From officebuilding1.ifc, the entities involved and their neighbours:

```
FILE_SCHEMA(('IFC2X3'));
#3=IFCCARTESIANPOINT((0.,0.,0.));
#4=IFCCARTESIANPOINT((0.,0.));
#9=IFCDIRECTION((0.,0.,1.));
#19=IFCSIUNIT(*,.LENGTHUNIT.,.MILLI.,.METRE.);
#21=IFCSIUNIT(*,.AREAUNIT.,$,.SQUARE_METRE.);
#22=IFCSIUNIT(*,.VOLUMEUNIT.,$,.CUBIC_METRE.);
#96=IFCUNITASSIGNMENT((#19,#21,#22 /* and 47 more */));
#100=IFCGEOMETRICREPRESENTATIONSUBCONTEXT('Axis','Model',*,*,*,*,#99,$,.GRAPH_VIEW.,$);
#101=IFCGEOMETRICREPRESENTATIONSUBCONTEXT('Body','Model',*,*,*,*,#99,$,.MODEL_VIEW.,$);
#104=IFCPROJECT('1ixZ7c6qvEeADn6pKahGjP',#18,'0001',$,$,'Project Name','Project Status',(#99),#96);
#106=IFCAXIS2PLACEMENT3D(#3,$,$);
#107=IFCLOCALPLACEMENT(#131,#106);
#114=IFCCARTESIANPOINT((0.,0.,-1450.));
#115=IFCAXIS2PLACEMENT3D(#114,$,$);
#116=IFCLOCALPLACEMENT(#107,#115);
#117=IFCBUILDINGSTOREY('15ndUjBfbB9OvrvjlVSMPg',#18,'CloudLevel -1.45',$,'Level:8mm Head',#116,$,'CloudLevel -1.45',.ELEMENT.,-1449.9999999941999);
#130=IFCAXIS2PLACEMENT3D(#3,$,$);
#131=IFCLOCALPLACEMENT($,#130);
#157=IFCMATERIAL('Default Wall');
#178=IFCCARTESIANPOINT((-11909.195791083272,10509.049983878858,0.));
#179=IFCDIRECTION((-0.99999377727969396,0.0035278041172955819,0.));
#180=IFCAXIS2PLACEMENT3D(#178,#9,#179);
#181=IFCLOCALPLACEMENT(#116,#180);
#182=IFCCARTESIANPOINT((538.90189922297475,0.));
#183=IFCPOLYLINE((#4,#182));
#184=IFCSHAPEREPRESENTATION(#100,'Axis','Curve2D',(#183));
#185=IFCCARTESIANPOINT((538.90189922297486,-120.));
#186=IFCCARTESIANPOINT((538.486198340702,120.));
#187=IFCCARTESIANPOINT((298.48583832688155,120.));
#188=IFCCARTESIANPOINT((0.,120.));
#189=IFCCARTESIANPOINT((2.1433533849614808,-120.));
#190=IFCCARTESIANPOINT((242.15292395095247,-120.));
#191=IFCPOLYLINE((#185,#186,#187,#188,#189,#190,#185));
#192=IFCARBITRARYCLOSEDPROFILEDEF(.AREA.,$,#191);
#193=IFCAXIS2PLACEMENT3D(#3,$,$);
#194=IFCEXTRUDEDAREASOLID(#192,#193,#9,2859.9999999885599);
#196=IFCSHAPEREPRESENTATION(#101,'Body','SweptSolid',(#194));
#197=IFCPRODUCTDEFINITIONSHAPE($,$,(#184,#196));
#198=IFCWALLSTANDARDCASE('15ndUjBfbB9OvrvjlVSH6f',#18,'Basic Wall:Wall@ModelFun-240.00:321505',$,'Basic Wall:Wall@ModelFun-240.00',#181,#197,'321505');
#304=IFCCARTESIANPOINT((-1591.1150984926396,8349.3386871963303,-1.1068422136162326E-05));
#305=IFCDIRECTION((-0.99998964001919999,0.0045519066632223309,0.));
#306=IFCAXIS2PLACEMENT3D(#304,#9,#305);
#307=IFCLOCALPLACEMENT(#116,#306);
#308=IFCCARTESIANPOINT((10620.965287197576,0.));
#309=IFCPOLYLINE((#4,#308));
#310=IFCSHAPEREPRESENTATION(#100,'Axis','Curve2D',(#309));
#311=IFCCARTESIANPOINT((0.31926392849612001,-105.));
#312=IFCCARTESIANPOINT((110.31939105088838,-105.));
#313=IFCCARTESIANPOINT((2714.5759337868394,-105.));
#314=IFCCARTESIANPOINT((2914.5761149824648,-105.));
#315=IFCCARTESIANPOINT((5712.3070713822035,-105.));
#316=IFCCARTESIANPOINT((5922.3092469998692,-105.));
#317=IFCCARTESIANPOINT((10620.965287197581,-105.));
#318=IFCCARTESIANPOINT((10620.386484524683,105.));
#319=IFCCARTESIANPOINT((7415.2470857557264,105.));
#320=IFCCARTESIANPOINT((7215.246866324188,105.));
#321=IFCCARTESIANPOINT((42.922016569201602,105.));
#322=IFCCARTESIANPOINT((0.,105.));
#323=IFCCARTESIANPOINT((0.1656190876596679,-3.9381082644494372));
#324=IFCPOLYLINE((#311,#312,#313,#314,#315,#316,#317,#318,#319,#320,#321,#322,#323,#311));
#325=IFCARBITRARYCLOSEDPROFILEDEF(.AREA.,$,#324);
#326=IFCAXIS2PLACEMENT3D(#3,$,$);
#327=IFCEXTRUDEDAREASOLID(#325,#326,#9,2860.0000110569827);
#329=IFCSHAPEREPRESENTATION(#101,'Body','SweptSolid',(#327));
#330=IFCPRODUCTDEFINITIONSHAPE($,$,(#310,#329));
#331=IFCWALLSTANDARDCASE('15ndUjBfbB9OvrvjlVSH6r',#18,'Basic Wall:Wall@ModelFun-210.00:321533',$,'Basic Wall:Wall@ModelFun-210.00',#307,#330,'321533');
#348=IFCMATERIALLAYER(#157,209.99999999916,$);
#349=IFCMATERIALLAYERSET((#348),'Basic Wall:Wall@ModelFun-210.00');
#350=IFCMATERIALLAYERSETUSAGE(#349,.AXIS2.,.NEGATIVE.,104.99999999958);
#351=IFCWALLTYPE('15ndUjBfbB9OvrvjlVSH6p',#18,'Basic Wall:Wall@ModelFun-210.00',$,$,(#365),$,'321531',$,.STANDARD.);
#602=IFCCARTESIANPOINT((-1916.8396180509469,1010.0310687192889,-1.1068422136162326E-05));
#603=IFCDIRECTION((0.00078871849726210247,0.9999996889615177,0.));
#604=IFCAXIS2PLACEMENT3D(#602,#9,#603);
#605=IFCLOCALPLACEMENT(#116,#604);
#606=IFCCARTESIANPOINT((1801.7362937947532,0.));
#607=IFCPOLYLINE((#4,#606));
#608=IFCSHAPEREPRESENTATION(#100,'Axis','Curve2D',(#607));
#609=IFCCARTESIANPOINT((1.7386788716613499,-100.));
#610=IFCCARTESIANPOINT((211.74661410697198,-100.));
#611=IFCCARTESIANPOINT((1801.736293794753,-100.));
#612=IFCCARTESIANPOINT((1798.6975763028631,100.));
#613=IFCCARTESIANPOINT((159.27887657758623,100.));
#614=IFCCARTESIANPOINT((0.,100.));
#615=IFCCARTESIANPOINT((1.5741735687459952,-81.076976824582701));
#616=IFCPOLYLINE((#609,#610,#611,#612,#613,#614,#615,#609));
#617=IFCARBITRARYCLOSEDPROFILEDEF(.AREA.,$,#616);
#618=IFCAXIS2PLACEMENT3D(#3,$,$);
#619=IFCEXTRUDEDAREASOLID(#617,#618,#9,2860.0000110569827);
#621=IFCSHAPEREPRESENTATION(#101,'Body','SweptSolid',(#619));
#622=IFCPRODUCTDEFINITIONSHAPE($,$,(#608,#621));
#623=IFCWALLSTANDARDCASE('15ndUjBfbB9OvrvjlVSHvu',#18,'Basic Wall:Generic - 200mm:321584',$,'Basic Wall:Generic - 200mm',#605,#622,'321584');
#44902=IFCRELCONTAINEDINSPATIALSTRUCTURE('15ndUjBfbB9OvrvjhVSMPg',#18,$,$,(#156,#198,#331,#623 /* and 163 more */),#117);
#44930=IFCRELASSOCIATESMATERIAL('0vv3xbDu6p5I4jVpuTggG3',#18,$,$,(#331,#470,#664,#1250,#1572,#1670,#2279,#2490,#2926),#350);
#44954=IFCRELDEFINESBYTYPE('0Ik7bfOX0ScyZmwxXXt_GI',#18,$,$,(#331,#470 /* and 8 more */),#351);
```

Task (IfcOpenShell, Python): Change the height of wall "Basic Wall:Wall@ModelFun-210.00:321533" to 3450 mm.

```python
import ifcopenshell
import ifcopenshell.geom
import ifcopenshell.util.representation
import ifcopenshell.util.shape

model = ifcopenshell.open("officebuilding1.ifc")
settings = ifcopenshell.geom.settings()


def volume(element):
    """Net volume in cubic metres, openings subtracted."""
    shape = ifcopenshell.geom.create_shape(settings, element)
    return ifcopenshell.util.shape.get_volume(shape.geometry)


wall = model.by_id(331)
before = volume(wall)

body = ifcopenshell.util.representation.get_representation(wall, "Model", "Body")
solid = body.Items[0]
old_height = solid.Depth
solid.Depth = 3450.0
after = volume(wall)

print(f"height {old_height:g} -> {solid.Depth:g}, volume {before:.3f} -> {after:.3f} m3")

model.write("officebuilding1_updated.ifc")
```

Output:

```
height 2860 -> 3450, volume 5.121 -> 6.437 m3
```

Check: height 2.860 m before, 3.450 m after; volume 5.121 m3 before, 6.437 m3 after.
